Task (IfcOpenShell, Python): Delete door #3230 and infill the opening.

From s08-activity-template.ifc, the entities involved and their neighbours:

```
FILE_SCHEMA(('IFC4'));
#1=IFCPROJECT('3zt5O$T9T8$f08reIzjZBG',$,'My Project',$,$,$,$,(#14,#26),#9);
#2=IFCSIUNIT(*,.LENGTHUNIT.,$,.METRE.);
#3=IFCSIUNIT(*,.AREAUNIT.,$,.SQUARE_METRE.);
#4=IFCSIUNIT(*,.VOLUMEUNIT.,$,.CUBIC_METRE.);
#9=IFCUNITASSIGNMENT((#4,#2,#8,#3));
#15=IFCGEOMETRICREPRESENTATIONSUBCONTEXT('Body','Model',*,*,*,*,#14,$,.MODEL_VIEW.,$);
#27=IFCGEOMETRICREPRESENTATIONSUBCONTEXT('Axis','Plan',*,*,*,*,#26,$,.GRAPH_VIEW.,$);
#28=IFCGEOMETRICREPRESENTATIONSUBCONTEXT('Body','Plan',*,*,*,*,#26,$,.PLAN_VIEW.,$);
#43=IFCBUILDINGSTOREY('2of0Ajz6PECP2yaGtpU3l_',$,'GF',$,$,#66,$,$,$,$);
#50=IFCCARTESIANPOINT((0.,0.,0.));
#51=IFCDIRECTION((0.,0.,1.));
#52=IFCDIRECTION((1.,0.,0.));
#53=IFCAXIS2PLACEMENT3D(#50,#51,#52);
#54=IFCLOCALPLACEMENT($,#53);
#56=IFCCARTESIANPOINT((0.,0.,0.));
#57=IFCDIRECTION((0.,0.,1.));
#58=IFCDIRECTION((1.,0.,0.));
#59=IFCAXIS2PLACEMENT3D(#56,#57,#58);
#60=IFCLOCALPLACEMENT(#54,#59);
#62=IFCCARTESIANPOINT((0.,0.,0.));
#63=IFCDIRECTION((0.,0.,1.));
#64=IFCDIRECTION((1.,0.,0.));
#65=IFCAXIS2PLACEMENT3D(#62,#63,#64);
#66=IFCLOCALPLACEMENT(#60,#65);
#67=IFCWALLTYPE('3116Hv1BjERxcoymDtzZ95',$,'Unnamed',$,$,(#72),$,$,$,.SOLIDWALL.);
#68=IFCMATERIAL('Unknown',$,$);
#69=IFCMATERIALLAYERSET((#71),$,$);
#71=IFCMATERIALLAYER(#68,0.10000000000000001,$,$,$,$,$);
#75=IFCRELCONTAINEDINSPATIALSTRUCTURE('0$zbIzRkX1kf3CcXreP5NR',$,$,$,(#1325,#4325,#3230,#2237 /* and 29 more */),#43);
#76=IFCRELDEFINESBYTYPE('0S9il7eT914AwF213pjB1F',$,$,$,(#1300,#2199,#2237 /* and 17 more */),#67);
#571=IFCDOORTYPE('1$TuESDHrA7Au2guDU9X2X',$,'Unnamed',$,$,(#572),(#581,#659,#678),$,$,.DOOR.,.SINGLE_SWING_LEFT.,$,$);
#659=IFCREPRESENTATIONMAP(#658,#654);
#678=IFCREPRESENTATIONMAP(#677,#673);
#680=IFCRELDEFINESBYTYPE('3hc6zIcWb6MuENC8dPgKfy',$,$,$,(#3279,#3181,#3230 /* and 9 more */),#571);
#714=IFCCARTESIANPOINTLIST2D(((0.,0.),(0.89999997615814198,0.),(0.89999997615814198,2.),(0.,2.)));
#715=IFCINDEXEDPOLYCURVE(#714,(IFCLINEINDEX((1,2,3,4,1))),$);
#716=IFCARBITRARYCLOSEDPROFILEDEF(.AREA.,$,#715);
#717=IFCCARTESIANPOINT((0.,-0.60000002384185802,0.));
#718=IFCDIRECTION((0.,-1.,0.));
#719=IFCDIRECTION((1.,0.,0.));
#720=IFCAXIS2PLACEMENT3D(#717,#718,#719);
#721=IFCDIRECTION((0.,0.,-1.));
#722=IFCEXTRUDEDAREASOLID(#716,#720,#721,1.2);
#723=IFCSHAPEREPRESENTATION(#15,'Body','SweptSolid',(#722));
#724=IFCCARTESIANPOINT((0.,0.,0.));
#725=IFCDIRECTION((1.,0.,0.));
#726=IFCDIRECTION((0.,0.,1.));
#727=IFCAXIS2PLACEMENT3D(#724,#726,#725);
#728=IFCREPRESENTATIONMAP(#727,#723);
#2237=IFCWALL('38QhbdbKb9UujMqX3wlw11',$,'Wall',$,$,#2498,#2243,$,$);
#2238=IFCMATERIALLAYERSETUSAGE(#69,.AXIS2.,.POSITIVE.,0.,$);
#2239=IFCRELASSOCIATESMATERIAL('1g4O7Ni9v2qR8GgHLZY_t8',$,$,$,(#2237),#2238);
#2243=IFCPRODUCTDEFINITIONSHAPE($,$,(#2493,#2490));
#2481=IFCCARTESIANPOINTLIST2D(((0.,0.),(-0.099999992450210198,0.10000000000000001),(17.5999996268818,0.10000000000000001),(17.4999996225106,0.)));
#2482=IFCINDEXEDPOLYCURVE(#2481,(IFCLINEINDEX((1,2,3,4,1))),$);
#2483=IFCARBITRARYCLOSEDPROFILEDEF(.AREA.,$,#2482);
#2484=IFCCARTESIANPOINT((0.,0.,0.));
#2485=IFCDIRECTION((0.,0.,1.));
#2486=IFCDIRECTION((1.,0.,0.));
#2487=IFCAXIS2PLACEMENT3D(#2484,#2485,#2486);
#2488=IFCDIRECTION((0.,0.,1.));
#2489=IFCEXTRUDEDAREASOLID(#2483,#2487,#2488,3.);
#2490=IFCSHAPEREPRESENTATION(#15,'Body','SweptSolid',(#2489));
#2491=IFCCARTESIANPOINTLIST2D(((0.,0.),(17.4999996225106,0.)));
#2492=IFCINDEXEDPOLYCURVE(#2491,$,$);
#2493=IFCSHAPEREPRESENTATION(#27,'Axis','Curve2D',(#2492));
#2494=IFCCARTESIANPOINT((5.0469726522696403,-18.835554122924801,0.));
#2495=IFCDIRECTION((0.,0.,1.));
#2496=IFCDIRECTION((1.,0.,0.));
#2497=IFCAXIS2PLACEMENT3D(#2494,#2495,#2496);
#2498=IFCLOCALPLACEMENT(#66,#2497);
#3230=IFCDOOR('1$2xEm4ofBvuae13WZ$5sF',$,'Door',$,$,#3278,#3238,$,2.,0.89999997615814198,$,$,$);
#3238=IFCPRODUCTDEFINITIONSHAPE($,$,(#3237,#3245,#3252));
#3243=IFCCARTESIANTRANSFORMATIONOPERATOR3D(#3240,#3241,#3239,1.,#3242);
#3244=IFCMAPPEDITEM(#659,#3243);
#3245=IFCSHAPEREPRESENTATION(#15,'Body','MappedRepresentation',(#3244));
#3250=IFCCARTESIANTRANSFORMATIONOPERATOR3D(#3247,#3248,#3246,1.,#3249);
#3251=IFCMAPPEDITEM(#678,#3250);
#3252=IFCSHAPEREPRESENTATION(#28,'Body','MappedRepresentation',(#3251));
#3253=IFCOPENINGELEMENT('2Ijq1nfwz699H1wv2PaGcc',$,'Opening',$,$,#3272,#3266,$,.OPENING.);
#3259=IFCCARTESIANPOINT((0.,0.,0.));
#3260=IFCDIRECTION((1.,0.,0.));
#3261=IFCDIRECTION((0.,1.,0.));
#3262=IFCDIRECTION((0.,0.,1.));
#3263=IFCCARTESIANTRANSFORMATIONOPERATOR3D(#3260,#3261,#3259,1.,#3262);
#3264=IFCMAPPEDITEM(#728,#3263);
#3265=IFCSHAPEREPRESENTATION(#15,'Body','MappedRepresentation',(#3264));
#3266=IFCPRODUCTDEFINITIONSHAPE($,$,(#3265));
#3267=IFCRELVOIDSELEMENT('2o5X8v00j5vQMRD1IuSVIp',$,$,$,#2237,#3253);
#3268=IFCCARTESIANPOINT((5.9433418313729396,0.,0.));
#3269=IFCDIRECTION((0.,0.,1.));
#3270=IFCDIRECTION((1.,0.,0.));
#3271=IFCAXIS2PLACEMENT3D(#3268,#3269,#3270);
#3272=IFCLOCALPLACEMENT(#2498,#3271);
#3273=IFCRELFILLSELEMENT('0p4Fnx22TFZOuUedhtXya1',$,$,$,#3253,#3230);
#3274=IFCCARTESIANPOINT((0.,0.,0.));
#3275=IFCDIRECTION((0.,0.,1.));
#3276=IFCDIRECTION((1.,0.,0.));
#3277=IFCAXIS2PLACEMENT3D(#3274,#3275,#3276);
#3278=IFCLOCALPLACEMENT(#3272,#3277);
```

```python
import ifcopenshell
import ifcopenshell.api.feature
import ifcopenshell.api.root
import ifcopenshell.geom
import ifcopenshell.util.shape

model = ifcopenshell.open("s08-activity-template.ifc")
settings = ifcopenshell.geom.settings()


def volume(element):
    """Net volume in cubic metres, openings subtracted."""
    shape = ifcopenshell.geom.create_shape(settings, element)
    return ifcopenshell.util.shape.get_volume(shape.geometry)


door = model.by_id(3230)
opening = door.FillsVoids[0].RelatingOpeningElement
wall = opening.VoidsElements[0].RelatingBuildingElement
before = volume(wall)

ifcopenshell.api.root.remove_product(model, product=door)
ifcopenshell.api.feature.remove_feature(model, feature=opening)

after = volume(wall)

print(f"wall volume {before:.3f} -> {after:.3f} m3")

model.write("s08-activity-template_edited.ifc")
```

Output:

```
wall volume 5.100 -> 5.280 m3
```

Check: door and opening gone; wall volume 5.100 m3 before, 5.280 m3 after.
